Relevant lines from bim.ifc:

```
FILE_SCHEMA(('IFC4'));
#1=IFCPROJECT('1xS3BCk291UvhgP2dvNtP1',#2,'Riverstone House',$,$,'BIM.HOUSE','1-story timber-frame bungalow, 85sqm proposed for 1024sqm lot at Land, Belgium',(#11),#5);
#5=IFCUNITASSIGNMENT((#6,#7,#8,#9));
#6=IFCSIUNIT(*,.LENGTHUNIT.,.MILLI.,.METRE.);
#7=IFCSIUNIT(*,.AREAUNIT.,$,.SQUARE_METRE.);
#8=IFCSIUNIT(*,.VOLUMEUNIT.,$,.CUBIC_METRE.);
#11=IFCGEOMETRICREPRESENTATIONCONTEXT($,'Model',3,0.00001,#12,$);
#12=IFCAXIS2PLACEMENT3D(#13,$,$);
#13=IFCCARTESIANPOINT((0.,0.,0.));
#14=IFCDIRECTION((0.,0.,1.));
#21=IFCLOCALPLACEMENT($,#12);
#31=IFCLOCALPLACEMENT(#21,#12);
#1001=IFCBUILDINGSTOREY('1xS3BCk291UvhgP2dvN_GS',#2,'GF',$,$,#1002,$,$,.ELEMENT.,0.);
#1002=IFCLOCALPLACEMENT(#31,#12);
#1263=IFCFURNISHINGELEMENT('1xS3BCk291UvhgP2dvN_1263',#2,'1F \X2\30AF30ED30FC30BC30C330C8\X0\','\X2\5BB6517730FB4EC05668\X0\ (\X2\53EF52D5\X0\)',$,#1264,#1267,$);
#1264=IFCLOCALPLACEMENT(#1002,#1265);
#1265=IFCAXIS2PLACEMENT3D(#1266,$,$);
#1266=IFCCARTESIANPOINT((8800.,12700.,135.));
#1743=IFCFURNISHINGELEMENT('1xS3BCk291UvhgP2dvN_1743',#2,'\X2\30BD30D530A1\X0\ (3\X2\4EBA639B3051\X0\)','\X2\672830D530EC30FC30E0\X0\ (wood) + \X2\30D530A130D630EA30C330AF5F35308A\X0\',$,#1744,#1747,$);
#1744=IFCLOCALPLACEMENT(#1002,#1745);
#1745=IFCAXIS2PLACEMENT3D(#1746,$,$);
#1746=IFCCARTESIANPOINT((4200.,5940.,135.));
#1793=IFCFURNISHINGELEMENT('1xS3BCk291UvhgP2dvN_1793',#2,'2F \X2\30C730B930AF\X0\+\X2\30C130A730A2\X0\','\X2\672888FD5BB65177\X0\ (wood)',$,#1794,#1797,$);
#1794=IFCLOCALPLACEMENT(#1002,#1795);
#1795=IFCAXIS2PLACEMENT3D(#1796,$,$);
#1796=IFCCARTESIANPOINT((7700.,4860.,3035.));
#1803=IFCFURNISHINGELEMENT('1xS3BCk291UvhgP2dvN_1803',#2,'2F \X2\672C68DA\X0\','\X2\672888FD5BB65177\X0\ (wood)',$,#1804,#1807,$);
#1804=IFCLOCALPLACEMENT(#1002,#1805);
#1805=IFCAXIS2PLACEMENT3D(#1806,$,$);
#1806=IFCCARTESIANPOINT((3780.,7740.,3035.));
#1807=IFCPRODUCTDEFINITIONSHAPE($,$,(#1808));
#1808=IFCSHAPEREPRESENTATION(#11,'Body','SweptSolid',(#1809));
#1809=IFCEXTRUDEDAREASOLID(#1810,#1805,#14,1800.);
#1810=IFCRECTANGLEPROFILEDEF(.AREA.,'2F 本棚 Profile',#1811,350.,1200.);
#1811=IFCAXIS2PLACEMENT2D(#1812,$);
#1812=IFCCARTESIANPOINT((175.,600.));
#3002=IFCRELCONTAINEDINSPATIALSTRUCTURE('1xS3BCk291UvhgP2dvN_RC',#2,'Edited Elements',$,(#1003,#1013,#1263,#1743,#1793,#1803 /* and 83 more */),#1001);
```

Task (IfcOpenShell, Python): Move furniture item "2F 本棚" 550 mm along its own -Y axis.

```python
import ifcopenshell
import ifcopenshell.api.geometry
import ifcopenshell.util.placement

model = ifcopenshell.open("bim.ifc")

item = model.by_id(1803)
matrix = ifcopenshell.util.placement.get_local_placement(item.ObjectPlacement)
matrix[:3, 3] -= matrix[:3, 1] * 550.0
ifcopenshell.api.geometry.edit_object_placement(model, product=item, matrix=matrix, is_si=False)

print(ifcopenshell.util.placement.get_local_placement(item.ObjectPlacement).round(3) + 0.0)

model.write("bim_edited.ifc")
```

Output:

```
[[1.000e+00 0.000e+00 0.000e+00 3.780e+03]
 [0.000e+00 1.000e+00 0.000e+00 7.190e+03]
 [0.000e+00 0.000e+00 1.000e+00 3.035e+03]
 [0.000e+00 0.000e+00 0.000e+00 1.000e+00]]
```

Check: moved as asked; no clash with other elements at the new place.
